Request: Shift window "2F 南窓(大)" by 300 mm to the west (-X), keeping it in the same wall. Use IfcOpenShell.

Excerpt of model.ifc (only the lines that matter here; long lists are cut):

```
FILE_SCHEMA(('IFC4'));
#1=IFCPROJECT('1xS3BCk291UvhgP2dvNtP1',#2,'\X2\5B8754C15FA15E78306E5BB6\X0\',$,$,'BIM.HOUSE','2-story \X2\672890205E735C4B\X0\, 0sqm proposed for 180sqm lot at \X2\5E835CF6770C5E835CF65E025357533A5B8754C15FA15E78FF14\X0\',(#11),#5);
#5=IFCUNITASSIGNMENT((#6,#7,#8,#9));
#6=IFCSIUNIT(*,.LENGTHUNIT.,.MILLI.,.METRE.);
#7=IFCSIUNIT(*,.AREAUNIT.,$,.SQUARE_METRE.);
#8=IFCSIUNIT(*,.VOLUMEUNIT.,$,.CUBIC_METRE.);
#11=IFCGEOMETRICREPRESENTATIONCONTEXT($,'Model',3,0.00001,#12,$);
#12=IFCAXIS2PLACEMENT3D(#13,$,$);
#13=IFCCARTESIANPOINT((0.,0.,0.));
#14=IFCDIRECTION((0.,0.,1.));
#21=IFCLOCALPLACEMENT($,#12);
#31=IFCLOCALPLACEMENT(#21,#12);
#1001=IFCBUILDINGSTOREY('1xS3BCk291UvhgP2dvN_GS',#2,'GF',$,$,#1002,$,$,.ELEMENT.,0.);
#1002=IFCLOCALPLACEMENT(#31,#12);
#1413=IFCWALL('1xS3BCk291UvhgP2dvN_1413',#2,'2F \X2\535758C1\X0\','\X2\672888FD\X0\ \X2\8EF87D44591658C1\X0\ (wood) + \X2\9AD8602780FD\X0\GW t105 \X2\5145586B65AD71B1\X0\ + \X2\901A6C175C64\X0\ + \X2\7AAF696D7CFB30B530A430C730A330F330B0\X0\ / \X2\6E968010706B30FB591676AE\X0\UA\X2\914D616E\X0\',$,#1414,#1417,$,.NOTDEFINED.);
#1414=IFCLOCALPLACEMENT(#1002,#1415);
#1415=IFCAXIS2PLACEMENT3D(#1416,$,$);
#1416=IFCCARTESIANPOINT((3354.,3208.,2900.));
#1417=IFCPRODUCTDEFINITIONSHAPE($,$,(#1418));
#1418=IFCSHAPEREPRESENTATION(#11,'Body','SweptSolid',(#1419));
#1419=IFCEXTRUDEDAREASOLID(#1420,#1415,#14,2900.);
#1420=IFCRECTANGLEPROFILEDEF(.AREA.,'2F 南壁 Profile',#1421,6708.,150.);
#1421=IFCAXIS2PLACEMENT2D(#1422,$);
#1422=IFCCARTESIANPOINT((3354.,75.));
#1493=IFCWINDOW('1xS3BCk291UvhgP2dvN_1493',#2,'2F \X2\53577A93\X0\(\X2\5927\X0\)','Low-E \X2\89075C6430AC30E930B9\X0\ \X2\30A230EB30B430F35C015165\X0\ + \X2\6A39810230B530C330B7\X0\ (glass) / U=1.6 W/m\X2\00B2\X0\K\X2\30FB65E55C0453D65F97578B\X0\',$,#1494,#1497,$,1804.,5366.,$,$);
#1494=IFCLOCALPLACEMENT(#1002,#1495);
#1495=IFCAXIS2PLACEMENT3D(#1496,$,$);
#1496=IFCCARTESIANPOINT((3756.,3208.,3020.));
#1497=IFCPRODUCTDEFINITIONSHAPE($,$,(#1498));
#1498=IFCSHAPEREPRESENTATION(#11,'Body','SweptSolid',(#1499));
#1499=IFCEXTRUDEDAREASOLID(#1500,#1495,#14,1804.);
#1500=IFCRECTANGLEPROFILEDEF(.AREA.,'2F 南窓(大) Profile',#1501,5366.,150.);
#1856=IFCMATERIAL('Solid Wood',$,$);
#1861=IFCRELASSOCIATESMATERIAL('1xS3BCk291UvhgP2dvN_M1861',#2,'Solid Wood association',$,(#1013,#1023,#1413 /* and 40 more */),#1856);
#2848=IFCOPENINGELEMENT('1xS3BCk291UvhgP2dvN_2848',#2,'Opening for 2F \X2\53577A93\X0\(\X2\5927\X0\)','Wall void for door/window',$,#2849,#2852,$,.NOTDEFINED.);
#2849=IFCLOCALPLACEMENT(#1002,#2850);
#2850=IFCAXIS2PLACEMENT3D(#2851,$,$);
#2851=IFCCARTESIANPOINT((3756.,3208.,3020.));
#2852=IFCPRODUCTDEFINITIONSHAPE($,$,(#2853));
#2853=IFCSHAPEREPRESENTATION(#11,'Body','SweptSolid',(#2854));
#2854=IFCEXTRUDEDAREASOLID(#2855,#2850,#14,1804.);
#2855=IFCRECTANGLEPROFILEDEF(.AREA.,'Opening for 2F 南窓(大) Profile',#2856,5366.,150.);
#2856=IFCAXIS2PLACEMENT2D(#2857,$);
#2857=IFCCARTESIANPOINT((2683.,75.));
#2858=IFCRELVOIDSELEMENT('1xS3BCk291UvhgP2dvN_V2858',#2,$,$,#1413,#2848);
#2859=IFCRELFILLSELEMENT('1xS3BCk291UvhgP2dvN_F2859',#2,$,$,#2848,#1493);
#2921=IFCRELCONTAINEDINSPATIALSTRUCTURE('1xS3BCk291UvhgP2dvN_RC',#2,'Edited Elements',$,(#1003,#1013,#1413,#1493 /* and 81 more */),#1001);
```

```python
import ifcopenshell
import ifcopenshell.api.geometry
import ifcopenshell.util.placement

model = ifcopenshell.open("model.ifc")

window = model.by_guid("1xS3BCk291UvhgP2dvN_1493")
opening = window.FillsVoids[0].RelatingOpeningElement
wall = opening.VoidsElements[0].RelatingBuildingElement

wall_matrix = ifcopenshell.util.placement.get_local_placement(wall.ObjectPlacement)
shift = wall_matrix[:3, 0] * -300.0
before = ifcopenshell.util.placement.get_local_placement(window.ObjectPlacement)[:3, 3].copy()

# The window is not placed relative to its opening, so move both.
for product in (opening, window):
    matrix = ifcopenshell.util.placement.get_local_placement(product.ObjectPlacement)
    matrix[:3, 3] += shift
    ifcopenshell.api.geometry.edit_object_placement(model, product=product, matrix=matrix, is_si=False)

after = ifcopenshell.util.placement.get_local_placement(window.ObjectPlacement)[:3, 3]
print("window moved by", (after - before).round(3) + 0.0)

model.write("model_updated.ifc")
```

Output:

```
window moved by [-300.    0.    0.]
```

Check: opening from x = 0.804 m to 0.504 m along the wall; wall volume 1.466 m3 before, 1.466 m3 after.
